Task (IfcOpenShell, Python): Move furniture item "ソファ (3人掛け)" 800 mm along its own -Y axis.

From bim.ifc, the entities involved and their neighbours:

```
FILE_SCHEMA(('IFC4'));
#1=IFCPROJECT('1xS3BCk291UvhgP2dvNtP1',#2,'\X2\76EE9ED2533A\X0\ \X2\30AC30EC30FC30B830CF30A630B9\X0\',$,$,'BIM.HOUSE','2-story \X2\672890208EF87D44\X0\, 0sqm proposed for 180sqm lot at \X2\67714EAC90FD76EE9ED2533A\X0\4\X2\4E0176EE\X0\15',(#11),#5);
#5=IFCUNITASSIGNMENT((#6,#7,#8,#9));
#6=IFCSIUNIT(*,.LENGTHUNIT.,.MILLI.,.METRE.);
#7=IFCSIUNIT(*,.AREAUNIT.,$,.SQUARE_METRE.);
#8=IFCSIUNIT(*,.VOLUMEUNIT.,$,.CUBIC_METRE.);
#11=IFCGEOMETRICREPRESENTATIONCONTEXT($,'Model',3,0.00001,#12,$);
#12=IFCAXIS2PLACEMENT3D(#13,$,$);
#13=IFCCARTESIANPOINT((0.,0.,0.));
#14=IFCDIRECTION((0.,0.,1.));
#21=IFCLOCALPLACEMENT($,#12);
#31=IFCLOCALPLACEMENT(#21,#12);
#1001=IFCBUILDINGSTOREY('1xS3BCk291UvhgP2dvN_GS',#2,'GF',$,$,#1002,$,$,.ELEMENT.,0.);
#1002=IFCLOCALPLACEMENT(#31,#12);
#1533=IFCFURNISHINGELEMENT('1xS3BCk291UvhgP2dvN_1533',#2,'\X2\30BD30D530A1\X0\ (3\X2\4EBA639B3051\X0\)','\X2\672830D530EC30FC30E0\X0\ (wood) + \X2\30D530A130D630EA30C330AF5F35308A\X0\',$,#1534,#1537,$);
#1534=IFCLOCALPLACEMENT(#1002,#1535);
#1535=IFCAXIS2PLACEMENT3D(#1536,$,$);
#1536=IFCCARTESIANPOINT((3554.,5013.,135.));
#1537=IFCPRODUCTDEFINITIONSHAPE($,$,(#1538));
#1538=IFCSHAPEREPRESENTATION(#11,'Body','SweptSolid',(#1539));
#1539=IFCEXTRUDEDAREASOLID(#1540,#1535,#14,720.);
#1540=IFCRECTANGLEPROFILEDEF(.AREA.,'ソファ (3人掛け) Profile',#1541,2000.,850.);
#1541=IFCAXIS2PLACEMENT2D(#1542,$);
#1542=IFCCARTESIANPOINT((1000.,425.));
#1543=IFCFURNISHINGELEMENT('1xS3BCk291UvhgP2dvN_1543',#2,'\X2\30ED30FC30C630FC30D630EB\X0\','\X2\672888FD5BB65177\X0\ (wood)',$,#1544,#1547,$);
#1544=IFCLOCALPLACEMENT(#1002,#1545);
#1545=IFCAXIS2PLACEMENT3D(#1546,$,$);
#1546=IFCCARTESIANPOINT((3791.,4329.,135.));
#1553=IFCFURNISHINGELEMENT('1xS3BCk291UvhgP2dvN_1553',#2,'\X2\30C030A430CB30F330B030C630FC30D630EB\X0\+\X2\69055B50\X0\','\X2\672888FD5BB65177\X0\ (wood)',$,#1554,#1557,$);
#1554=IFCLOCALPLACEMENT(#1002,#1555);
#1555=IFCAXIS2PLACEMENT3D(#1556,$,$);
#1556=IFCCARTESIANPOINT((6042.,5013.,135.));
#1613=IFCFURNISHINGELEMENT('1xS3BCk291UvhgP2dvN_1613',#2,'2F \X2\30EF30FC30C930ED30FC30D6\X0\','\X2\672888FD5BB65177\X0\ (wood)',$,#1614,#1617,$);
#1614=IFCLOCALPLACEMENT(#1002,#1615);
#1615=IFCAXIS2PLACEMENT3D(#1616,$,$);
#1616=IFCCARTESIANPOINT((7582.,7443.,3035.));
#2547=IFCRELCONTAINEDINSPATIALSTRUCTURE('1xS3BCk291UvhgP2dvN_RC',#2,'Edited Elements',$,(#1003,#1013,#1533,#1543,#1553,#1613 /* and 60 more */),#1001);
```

```python
import ifcopenshell
import ifcopenshell.api.geometry
import ifcopenshell.util.placement
import ifcopenshell.util.unit

model = ifcopenshell.open("bim.ifc")
unit_scale = ifcopenshell.util.unit.calculate_unit_scale(model)

item = model.by_id(1533)
matrix = ifcopenshell.util.placement.get_local_placement(item.ObjectPlacement)
matrix[:3, 3] -= matrix[:3, 1] * 0.8 / unit_scale
ifcopenshell.api.geometry.edit_object_placement(model, product=item, matrix=matrix, is_si=False)

print(ifcopenshell.util.placement.get_local_placement(item.ObjectPlacement).round(3) + 0.0)

model.write("bim_v2.ifc")
```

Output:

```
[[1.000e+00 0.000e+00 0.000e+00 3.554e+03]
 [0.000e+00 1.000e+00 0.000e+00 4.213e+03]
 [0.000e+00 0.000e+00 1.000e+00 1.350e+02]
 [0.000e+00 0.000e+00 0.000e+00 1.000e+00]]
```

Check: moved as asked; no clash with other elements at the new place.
